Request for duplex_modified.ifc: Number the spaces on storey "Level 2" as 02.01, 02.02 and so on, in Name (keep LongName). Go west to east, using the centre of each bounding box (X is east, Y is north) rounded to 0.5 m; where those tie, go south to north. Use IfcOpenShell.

First a look at what the model holds.

```python
import ifcopenshell
import ifcopenshell.util.element
import ifcopenshell.util.placement

model = ifcopenshell.open("duplex_modified.ifc")
print(model.schema)
storey = next(s for s in model.by_type("IfcBuildingStorey") if s.Name == "Level 2")
spaces = [e for e in ifcopenshell.util.element.get_decomposition(storey) if e.is_a("IfcSpace")]
for e in sorted(spaces, key=lambda e: e.id()):
    origin = ifcopenshell.util.placement.get_local_placement(e.ObjectPlacement)[:3, 3]
    print(e.id(), e.Name, e.LongName, origin.round(2) + 0.0, sep=" | ")
```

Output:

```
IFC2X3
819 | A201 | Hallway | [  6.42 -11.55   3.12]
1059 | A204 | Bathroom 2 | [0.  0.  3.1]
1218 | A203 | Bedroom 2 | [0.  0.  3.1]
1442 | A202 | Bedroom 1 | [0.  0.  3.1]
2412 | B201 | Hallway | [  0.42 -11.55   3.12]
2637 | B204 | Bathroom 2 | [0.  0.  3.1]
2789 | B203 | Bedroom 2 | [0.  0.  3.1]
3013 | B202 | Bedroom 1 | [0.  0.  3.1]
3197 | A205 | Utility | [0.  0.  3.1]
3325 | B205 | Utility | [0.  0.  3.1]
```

```python
import ifcopenshell
import ifcopenshell.geom
import ifcopenshell.util.element
import ifcopenshell.util.shape

model = ifcopenshell.open("duplex_modified.ifc")
settings = ifcopenshell.geom.settings()
settings.set("use-world-coords", True)


def centre(element):
    shape = ifcopenshell.geom.create_shape(settings, element)
    return ifcopenshell.util.shape.get_bbox_centroid(shape.geometry)


storey = next(s for s in model.by_type("IfcBuildingStorey") if s.Name == "Level 2")
spaces = [e for e in ifcopenshell.util.element.get_decomposition(storey) if e.is_a("IfcSpace")]

# Insertion points can sit at a corner or the storey origin, so sort by the geometry (in metres).
centres = {e: centre(e) for e in spaces}
spaces.sort(key=lambda e: (round(centres[e][0] / 0.5), centres[e][1]))

for i, e in enumerate(spaces, start=1):
    number = f"02.{i:02d}"
    e.Name = number
    print(e.id(), number)

model.write("duplex_modified-out.ifc")
```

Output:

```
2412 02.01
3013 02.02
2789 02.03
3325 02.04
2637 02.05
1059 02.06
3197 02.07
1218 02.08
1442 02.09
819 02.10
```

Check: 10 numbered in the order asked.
